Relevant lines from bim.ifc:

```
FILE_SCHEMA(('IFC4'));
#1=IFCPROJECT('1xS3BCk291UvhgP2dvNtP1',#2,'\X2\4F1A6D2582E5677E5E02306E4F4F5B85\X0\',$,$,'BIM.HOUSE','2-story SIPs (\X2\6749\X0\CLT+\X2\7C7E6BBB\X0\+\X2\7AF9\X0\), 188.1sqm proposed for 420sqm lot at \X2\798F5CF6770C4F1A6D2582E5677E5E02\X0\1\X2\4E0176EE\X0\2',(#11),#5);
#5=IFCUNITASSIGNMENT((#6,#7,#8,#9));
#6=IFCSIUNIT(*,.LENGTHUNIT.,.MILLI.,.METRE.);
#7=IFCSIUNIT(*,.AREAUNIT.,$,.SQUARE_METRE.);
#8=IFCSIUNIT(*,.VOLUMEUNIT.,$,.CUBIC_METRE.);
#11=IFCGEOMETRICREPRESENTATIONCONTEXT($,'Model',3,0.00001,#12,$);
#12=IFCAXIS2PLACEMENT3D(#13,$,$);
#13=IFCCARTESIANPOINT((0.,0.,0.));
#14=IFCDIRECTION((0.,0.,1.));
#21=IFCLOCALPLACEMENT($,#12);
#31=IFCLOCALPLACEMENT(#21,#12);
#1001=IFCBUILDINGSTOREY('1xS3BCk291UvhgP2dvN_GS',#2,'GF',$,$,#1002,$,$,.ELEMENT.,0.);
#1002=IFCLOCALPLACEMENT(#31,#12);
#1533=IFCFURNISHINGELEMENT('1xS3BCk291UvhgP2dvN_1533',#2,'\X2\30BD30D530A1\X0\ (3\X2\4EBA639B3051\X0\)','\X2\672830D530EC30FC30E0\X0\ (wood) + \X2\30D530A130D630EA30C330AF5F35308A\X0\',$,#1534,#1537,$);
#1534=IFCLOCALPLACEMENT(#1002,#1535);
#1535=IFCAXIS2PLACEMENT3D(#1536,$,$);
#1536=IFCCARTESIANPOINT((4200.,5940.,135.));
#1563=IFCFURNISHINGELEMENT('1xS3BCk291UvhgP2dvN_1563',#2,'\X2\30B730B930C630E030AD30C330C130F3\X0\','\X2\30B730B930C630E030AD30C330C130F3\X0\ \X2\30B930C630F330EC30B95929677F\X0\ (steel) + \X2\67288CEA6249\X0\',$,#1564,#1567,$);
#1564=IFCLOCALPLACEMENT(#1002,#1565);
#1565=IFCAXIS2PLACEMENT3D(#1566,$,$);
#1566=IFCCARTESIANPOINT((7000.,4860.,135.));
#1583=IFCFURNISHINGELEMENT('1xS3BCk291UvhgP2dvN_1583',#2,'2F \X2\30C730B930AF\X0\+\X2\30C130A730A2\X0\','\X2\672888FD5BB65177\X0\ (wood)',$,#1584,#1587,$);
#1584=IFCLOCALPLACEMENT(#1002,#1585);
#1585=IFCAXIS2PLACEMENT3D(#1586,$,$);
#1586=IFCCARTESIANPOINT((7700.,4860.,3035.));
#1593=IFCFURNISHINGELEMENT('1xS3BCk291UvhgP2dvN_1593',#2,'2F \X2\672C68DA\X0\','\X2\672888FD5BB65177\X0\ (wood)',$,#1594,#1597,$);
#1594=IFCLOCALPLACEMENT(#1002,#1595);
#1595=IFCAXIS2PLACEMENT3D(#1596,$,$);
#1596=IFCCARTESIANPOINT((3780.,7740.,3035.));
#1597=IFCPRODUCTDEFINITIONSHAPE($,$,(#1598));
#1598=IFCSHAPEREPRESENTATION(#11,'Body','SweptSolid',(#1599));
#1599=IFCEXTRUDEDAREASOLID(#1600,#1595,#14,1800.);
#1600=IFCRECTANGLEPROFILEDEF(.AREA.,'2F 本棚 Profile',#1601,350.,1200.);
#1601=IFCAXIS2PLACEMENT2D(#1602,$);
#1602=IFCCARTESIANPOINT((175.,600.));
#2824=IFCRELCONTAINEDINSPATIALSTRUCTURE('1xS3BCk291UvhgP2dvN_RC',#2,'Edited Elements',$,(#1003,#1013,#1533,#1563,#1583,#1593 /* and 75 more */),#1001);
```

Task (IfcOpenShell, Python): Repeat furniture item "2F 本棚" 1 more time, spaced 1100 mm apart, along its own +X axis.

```python
import ifcopenshell
import ifcopenshell.api.geometry
import ifcopenshell.api.root
import ifcopenshell.util.element
import ifcopenshell.util.placement
import ifcopenshell.util.unit

model = ifcopenshell.open("bim.ifc")
unit_scale = ifcopenshell.util.unit.calculate_unit_scale(model)


def reuse_history(source, copy):
    """copy_class also copies each property set's owner history, people and application; keep the originals."""
    for rel in copy.IsDefinedBy:
        if rel.is_a("IfcRelDefinesByProperties") and (history := rel.RelatingPropertyDefinition.OwnerHistory):
            rel.RelatingPropertyDefinition.OwnerHistory = source.OwnerHistory
            ifcopenshell.util.element.remove_deep2(model, history)


source = model.by_guid("1xS3BCk291UvhgP2dvN_1593")
base = ifcopenshell.util.placement.get_local_placement(source.ObjectPlacement)
step = base[:3, 0] * 1.1 / unit_scale

for i in range(1, 2):
    copy = ifcopenshell.api.root.copy_class(model, product=source)
    copy.Representation = ifcopenshell.util.element.copy_deep(
        model, source.Representation, exclude=["IfcGeometricRepresentationContext", "IfcRepresentationMap"]
    )
    reuse_history(source, copy)
    matrix = base.copy()
    matrix[:3, 3] += i * step
    print("added at", matrix[:3, 3].round(3) + 0.0)
    ifcopenshell.api.geometry.edit_object_placement(model, product=copy, matrix=matrix, is_si=False)

model.write("bim_edited.ifc")
```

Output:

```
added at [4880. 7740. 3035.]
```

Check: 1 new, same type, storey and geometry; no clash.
